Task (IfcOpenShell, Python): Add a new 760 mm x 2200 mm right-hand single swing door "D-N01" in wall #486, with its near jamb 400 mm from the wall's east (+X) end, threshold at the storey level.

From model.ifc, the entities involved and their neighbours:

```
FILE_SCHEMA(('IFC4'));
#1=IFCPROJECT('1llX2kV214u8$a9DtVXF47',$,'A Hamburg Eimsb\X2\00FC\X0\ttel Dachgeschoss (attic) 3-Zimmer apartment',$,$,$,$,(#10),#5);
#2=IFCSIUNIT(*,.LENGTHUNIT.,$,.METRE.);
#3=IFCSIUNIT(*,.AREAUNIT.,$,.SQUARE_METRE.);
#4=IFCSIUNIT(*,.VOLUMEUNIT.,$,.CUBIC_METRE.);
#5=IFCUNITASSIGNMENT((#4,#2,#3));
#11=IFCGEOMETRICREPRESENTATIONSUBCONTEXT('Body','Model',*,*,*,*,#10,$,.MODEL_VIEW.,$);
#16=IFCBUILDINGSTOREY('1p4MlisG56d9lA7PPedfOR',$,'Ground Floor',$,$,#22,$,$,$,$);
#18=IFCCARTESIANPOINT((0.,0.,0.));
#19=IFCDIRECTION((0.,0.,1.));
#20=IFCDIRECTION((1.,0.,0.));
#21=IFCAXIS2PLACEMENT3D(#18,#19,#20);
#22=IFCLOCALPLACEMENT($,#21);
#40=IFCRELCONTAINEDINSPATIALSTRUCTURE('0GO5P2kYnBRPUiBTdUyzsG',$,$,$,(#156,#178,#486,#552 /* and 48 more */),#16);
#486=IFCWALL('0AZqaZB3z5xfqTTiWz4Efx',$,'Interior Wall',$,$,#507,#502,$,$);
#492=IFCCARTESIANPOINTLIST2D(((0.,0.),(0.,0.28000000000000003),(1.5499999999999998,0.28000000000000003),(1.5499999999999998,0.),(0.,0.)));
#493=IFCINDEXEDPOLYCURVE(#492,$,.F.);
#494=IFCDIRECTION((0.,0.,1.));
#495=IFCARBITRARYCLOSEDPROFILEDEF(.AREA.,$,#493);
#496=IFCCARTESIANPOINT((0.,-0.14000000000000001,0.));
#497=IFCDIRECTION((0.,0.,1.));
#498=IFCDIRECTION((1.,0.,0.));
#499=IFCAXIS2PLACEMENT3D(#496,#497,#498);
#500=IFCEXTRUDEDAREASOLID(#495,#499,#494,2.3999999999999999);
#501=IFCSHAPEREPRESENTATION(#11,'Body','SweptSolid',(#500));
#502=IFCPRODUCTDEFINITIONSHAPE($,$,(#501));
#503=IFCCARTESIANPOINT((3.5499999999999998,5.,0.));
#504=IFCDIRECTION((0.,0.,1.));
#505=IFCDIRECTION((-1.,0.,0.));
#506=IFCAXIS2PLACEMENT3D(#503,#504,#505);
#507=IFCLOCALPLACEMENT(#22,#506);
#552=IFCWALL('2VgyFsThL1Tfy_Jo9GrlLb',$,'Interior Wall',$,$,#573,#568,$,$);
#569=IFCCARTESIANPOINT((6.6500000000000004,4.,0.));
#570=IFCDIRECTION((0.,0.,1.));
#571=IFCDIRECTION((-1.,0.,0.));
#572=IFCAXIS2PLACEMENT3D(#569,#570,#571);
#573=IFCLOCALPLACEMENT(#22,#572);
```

```python
import numpy as np
import ifcopenshell
import ifcopenshell.api.feature
import ifcopenshell.api.geometry
import ifcopenshell.api.root
import ifcopenshell.api.spatial
import ifcopenshell.geom
import ifcopenshell.util.element
import ifcopenshell.util.placement
import ifcopenshell.util.representation
import ifcopenshell.util.shape
import ifcopenshell.util.unit

model = ifcopenshell.open("model.ifc")
unit_scale = ifcopenshell.util.unit.calculate_unit_scale(model)
settings = ifcopenshell.geom.settings()


def volume(element):
    """Net volume in cubic metres, openings subtracted."""
    shape = ifcopenshell.geom.create_shape(settings, element)
    return ifcopenshell.util.shape.get_volume(shape.geometry)


wall = model.by_id(486)
storey = ifcopenshell.util.element.get_container(wall, ifc_class="IfcBuildingStorey")
context = ifcopenshell.util.representation.get_context(model, "Model", "Body", "MODEL_VIEW")
before = volume(wall)

width, height, from_end, sill = 0.76, 2.2, 0.4, 0.0  # metres

# The wall runs along its own X axis, and the end named is its -X end.
wall_shape = ifcopenshell.geom.create_shape(settings, wall)
x, y, z = ifcopenshell.util.shape.get_vertices(wall_shape.geometry).T
start = x.min() + from_end
face, thickness = float(y.min()), float(y.max() - y.min())
wall_matrix = ifcopenshell.util.placement.get_local_placement(wall.ObjectPlacement)
level = ifcopenshell.util.placement.get_local_placement(storey.ObjectPlacement)[2, 3]


def in_wall(x, y):
    """Placement at x, y metres in the wall's axes, at sill height."""
    matrix = wall_matrix.copy()
    matrix[:, 3] = wall_matrix @ np.array([x / unit_scale, y / unit_scale, 0.0, 1.0])
    matrix[2, 3] = level + sill / unit_scale
    return matrix


# Opening: a box that overshoots both wall faces by 50 mm.
opening = ifcopenshell.api.root.create_entity(model, ifc_class="IfcOpeningElement", predefined_type="OPENING")
box = ifcopenshell.api.geometry.add_wall_representation(
    model, context=context, length=width, height=height, thickness=thickness + 0.1
)
ifcopenshell.api.geometry.assign_representation(model, product=opening, representation=box)
ifcopenshell.api.geometry.edit_object_placement(model, product=opening, matrix=in_wall(start, face - 0.05), is_si=False)
ifcopenshell.api.feature.add_feature(model, feature=opening, element=wall)

door = ifcopenshell.api.root.create_entity(model, ifc_class="IfcDoor", name="D-N01", predefined_type="DOOR")
door.OverallWidth, door.OverallHeight = width / unit_scale, height / unit_scale
door.OperationType = "SINGLE_SWING_RIGHT"
body = ifcopenshell.api.geometry.add_door_representation(
    model,
    context=context,
    overall_width=door.OverallWidth,
    overall_height=door.OverallHeight,
    operation_type="SINGLE_SWING_RIGHT",
    lining_properties={"LiningDepth": thickness / unit_scale, "ThresholdDepth": thickness / unit_scale},
)
ifcopenshell.api.geometry.assign_representation(model, product=door, representation=body)
ifcopenshell.api.spatial.assign_container(model, products=[door], relating_structure=storey)
ifcopenshell.api.feature.add_filling(model, opening=opening, element=door)

# The lining spans the wall, so the door starts at the wall face.
ifcopenshell.api.geometry.edit_object_placement(model, product=door, matrix=in_wall(start, face), is_si=False)

after = volume(wall)

print(f"wall volume {before:.3f} -> {after:.3f} m3")

model.write("model_v2.ifc")
```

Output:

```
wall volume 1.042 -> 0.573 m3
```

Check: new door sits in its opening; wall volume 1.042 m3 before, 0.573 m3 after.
